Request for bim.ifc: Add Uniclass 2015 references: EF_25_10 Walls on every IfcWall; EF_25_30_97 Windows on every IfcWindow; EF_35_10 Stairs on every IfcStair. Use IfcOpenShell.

First a look at what the model holds.

```python
import ifcopenshell

model = ifcopenshell.open("bim.ifc")
print(model.schema)
print("classifications:", [c.Name for c in model.by_type("IfcClassification")])
for ifc_class in ("IfcDoor", "IfcRoof", "IfcStair", "IfcWall", "IfcWindow"):
    print(ifc_class, len(model.by_type(ifc_class)))
```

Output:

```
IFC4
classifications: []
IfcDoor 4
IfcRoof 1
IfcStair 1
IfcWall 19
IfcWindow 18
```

```python
import ifcopenshell
import ifcopenshell.api.classification

model = ifcopenshell.open("bim.ifc")

system = ifcopenshell.api.classification.add_classification(model, classification="Uniclass 2015")

codes = {
    "IfcWall": ("EF_25_10", "Walls"),
    "IfcWindow": ("EF_25_30_97", "Windows"),
    "IfcStair": ("EF_35_10", "Stairs"),
}
for ifc_class, (code, name) in codes.items():
    products = model.by_type(ifc_class)
    ifcopenshell.api.classification.add_reference(
        model, products=products, classification=system, identification=code, name=name
    )
    print(code, len(products))

model.write("bim_edited.ifc")
```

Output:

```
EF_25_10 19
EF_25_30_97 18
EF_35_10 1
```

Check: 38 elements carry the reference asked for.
